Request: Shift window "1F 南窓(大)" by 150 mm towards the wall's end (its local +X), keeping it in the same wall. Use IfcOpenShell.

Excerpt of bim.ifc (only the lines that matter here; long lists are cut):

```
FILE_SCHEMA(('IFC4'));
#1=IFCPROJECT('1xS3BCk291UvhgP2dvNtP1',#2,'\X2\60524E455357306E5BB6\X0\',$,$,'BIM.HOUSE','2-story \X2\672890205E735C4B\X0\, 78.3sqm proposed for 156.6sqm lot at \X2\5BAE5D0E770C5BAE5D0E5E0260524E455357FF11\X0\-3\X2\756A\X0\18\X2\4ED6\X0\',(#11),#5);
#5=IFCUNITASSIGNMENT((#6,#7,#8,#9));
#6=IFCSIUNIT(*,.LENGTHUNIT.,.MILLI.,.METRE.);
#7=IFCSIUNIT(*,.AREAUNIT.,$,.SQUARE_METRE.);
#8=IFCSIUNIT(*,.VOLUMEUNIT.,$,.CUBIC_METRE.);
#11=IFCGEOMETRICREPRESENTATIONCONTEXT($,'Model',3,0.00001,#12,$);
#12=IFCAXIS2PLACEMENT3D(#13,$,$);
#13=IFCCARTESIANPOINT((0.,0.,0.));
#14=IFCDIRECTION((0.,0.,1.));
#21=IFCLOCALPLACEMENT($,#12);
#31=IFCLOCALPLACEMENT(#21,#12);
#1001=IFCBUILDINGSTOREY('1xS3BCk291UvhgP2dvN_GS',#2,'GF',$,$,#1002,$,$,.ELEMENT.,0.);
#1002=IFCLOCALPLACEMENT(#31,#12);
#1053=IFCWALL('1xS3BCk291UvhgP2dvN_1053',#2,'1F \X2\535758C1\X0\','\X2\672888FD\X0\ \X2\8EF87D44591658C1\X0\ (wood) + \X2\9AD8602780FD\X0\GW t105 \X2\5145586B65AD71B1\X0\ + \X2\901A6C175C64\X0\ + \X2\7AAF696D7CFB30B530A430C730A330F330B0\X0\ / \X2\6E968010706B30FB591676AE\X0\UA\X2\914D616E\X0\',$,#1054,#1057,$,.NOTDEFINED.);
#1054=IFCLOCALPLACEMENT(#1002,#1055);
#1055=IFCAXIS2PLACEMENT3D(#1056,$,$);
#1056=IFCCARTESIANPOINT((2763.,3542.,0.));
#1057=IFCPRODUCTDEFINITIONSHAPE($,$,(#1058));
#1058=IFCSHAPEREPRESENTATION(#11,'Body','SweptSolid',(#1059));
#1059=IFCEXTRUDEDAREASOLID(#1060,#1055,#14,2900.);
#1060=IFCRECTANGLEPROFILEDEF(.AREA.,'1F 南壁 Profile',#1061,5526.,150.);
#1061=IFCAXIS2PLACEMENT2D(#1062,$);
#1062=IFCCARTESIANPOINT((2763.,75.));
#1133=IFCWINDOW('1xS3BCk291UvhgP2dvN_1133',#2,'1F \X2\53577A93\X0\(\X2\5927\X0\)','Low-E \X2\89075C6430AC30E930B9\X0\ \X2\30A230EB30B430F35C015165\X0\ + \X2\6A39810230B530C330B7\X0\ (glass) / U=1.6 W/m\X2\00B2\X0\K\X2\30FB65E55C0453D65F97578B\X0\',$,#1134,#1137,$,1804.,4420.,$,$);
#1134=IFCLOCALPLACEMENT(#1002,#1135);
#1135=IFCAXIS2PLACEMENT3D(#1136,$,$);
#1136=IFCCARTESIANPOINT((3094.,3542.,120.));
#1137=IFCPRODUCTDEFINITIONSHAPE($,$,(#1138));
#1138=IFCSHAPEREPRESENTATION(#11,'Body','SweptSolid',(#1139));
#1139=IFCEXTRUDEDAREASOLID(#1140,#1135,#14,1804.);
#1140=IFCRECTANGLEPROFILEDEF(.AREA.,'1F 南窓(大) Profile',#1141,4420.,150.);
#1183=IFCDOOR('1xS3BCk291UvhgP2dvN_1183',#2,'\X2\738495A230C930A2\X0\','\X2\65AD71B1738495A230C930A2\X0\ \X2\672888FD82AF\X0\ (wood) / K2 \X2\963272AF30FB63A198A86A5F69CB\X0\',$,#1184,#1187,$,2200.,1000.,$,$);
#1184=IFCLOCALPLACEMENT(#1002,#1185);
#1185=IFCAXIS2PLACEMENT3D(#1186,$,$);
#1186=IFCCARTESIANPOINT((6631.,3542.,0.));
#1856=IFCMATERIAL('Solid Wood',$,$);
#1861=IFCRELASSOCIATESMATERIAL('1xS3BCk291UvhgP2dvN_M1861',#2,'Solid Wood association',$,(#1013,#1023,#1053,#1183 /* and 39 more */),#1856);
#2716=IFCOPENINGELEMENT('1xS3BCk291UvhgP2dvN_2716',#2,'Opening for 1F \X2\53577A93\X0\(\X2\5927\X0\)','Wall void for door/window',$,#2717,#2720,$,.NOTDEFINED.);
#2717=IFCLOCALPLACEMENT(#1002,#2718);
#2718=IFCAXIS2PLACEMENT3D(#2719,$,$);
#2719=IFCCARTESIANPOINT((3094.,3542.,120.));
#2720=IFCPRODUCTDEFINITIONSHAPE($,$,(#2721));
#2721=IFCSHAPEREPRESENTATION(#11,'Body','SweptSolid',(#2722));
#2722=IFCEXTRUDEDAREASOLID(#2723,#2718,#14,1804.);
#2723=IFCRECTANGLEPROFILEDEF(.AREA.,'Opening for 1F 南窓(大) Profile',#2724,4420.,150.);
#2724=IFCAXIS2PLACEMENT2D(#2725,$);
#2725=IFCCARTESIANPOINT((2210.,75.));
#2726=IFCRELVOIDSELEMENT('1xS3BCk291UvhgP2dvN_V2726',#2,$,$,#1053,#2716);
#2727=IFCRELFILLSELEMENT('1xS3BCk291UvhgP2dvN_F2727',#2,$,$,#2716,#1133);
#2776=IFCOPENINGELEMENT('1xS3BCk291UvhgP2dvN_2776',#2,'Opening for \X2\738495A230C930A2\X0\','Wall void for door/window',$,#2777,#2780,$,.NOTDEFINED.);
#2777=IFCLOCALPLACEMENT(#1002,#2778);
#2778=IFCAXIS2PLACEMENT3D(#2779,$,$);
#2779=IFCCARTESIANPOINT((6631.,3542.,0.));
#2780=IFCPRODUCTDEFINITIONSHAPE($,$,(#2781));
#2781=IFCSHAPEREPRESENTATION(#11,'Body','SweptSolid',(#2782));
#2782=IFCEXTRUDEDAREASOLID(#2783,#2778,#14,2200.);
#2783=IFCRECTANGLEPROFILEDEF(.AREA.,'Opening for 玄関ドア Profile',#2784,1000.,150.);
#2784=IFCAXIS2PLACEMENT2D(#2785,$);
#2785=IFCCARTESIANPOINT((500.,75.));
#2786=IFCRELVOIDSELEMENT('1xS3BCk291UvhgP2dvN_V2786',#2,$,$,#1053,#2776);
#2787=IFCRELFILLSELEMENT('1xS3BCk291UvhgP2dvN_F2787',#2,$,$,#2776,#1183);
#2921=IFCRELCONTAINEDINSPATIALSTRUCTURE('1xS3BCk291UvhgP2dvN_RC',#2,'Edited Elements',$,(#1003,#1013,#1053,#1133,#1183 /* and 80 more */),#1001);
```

```python
import ifcopenshell
import ifcopenshell.api.geometry
import ifcopenshell.util.placement
import ifcopenshell.util.unit

model = ifcopenshell.open("bim.ifc")
unit_scale = ifcopenshell.util.unit.calculate_unit_scale(model)

window = model.by_id(1133)
opening = window.FillsVoids[0].RelatingOpeningElement
wall = opening.VoidsElements[0].RelatingBuildingElement

wall_matrix = ifcopenshell.util.placement.get_local_placement(wall.ObjectPlacement)
shift = wall_matrix[:3, 0] * 0.15 / unit_scale
before = ifcopenshell.util.placement.get_local_placement(window.ObjectPlacement)[:3, 3].copy()

# The window is not placed relative to its opening, so move both.
for product in (opening, window):
    matrix = ifcopenshell.util.placement.get_local_placement(product.ObjectPlacement)
    matrix[:3, 3] += shift
    ifcopenshell.api.geometry.edit_object_placement(model, product=product, matrix=matrix, is_si=False)

after = ifcopenshell.util.placement.get_local_placement(window.ObjectPlacement)[:3, 3]
print("window moved by", (after - before).round(3) + 0.0)

model.write("bim_v2.ifc")
```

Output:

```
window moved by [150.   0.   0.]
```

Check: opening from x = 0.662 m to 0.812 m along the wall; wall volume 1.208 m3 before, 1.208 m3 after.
